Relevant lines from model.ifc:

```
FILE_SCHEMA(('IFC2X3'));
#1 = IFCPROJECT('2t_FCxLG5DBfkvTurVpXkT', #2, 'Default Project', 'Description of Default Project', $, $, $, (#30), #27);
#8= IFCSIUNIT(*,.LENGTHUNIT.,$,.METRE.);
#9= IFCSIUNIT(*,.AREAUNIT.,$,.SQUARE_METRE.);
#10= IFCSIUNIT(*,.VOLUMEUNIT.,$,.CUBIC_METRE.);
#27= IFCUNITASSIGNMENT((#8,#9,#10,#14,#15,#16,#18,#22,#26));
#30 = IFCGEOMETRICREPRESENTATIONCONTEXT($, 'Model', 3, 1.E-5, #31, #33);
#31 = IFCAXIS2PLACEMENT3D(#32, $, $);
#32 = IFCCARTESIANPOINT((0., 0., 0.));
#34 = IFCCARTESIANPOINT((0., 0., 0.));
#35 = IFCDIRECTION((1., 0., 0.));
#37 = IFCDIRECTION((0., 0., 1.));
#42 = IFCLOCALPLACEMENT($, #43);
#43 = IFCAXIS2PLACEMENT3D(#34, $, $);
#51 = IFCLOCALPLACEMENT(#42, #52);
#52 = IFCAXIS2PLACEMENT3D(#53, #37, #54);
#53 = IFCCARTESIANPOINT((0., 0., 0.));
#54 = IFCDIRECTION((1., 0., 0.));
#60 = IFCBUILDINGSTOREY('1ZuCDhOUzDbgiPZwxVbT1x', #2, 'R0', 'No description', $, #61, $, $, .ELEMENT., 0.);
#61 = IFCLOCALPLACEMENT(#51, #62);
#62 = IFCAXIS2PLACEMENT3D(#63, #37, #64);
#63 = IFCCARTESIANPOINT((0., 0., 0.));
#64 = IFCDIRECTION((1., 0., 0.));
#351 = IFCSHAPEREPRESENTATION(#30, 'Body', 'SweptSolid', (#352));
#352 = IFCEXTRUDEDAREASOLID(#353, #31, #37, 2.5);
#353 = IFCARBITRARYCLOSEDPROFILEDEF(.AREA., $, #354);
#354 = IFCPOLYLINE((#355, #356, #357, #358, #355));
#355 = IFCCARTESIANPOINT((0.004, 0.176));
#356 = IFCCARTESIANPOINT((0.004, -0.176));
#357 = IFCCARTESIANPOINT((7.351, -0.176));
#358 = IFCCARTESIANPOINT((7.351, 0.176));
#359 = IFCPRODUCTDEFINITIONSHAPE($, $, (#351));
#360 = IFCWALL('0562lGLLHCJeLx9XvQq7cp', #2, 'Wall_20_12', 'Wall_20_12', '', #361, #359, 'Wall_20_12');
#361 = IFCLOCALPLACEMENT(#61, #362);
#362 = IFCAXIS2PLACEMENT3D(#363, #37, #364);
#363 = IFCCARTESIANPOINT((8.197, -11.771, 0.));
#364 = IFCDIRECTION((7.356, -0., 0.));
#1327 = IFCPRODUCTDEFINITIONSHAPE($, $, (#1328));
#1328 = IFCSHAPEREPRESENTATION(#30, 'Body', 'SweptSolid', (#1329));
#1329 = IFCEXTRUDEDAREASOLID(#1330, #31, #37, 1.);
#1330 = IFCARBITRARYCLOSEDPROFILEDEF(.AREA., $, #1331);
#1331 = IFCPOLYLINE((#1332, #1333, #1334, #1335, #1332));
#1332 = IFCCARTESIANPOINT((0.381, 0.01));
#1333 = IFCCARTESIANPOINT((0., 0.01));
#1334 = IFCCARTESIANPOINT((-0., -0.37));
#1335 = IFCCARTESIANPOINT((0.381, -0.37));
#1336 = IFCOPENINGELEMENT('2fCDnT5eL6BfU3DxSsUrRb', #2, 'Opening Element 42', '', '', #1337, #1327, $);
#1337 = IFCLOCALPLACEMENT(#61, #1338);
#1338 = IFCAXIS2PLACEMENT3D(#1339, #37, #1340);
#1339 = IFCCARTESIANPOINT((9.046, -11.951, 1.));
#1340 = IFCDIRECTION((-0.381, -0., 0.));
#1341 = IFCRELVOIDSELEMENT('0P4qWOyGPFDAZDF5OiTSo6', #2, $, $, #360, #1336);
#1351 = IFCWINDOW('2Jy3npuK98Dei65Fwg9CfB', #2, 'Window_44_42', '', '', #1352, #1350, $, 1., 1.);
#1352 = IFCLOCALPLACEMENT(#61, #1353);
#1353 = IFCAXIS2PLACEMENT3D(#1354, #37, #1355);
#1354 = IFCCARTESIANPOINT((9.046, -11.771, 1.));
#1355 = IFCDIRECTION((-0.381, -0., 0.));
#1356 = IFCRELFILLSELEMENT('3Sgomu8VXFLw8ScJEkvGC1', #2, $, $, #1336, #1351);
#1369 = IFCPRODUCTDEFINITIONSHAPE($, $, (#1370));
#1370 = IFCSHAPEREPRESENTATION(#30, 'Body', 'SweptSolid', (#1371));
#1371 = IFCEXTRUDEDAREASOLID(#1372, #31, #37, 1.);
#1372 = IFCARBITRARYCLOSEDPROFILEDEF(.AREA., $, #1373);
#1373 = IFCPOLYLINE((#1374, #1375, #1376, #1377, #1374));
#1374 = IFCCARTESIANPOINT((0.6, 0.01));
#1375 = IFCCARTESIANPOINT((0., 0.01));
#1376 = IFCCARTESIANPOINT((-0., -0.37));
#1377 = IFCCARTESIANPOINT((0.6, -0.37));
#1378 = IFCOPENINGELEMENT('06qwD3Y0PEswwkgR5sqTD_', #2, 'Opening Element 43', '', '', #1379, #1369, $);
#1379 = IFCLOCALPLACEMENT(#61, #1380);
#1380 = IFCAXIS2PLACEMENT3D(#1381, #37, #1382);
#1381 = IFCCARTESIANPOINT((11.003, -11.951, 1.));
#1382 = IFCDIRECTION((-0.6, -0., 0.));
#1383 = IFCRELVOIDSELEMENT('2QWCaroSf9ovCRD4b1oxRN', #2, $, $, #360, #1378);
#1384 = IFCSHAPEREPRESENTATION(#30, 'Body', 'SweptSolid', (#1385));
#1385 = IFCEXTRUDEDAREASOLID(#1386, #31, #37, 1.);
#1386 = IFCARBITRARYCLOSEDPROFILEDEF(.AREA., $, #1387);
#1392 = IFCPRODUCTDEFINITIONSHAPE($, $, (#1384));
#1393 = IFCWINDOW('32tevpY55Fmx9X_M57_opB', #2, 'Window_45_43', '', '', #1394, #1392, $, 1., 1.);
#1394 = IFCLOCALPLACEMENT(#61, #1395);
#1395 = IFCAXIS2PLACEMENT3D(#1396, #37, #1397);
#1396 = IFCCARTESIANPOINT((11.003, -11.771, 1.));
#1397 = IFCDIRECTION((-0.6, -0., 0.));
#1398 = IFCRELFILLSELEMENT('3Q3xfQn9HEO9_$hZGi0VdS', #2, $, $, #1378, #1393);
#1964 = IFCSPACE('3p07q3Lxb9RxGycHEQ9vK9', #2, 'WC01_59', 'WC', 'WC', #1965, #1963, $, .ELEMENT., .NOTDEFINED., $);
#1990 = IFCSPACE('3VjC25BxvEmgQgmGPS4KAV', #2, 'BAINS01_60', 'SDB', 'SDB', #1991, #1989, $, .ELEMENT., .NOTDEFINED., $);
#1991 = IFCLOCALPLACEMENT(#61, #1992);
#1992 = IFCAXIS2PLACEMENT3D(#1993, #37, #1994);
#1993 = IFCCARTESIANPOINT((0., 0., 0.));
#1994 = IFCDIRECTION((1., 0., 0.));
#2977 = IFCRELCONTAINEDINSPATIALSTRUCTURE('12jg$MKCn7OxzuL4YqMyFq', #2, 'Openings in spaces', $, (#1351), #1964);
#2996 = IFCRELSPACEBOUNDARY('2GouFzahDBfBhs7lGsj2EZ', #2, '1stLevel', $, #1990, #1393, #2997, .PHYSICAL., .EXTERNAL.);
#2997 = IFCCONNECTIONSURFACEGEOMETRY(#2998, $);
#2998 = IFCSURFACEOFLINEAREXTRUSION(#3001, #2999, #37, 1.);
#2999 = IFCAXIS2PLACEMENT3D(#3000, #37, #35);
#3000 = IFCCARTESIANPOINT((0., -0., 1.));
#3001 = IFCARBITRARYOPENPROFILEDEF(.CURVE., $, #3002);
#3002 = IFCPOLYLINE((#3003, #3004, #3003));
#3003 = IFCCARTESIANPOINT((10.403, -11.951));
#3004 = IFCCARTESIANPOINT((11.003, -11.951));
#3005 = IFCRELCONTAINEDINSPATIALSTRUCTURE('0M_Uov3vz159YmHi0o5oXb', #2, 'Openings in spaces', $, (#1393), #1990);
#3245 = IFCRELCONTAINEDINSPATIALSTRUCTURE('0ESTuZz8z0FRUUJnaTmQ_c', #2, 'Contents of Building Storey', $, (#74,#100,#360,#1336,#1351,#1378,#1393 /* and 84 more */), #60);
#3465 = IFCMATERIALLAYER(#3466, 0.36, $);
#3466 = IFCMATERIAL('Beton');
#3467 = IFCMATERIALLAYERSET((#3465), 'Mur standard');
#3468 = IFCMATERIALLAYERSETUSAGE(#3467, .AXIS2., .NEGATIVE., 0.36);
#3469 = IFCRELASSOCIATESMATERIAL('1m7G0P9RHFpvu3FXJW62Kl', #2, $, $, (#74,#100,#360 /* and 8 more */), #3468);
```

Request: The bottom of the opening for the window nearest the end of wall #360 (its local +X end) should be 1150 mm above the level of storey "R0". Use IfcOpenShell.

```python
import numpy as np
import ifcopenshell
import ifcopenshell.api.geometry
import ifcopenshell.geom
import ifcopenshell.util.element
import ifcopenshell.util.placement
import ifcopenshell.util.shape
import ifcopenshell.util.unit

model = ifcopenshell.open("model.ifc")
unit_scale = ifcopenshell.util.unit.calculate_unit_scale(model)

window = model.by_id(1393)
opening = window.FillsVoids[0].RelatingOpeningElement
storey = ifcopenshell.util.element.get_container(window, ifc_class="IfcBuildingStorey")
level = ifcopenshell.util.placement.get_local_placement(storey.ObjectPlacement)[2, 3]

# The opening's origin need not be at the sill, so measure its lowest point.
shape = ifcopenshell.geom.create_shape(ifcopenshell.geom.settings(), opening)
bottom = ifcopenshell.util.shape.get_shape_bottom_elevation(shape, shape.geometry) / unit_scale
dz = level + 1.15 - bottom

shift = np.array([0.0, 0.0, dz])
# The window is not placed relative to its opening, so move both.
for product in (opening, window):
    matrix = ifcopenshell.util.placement.get_local_placement(product.ObjectPlacement)
    matrix[:3, 3] += shift
    ifcopenshell.api.geometry.edit_object_placement(model, product=product, matrix=matrix, is_si=False)

# Space boundary surfaces are stored in each space's coordinates; move them too.
for rel in window.ProvidesBoundaries:
    if not rel.ConnectionGeometry:
        continue
    surface = rel.ConnectionGeometry.SurfaceOnRelatingElement
    space_matrix = ifcopenshell.util.placement.get_local_placement(rel.RelatingSpace.ObjectPlacement)
    point = np.array(surface.Position.Location.Coordinates) + space_matrix[:3, :3].T @ shift
    surface.Position = model.createIfcAxis2Placement3D(
        model.createIfcCartesianPoint(point.tolist()), surface.Position.Axis, surface.Position.RefDirection
    )

print(f"moved by {dz * unit_scale:+.3f} m")

model.write("model_edited.ifc")
```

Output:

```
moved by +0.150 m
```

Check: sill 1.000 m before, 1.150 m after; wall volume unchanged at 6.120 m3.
